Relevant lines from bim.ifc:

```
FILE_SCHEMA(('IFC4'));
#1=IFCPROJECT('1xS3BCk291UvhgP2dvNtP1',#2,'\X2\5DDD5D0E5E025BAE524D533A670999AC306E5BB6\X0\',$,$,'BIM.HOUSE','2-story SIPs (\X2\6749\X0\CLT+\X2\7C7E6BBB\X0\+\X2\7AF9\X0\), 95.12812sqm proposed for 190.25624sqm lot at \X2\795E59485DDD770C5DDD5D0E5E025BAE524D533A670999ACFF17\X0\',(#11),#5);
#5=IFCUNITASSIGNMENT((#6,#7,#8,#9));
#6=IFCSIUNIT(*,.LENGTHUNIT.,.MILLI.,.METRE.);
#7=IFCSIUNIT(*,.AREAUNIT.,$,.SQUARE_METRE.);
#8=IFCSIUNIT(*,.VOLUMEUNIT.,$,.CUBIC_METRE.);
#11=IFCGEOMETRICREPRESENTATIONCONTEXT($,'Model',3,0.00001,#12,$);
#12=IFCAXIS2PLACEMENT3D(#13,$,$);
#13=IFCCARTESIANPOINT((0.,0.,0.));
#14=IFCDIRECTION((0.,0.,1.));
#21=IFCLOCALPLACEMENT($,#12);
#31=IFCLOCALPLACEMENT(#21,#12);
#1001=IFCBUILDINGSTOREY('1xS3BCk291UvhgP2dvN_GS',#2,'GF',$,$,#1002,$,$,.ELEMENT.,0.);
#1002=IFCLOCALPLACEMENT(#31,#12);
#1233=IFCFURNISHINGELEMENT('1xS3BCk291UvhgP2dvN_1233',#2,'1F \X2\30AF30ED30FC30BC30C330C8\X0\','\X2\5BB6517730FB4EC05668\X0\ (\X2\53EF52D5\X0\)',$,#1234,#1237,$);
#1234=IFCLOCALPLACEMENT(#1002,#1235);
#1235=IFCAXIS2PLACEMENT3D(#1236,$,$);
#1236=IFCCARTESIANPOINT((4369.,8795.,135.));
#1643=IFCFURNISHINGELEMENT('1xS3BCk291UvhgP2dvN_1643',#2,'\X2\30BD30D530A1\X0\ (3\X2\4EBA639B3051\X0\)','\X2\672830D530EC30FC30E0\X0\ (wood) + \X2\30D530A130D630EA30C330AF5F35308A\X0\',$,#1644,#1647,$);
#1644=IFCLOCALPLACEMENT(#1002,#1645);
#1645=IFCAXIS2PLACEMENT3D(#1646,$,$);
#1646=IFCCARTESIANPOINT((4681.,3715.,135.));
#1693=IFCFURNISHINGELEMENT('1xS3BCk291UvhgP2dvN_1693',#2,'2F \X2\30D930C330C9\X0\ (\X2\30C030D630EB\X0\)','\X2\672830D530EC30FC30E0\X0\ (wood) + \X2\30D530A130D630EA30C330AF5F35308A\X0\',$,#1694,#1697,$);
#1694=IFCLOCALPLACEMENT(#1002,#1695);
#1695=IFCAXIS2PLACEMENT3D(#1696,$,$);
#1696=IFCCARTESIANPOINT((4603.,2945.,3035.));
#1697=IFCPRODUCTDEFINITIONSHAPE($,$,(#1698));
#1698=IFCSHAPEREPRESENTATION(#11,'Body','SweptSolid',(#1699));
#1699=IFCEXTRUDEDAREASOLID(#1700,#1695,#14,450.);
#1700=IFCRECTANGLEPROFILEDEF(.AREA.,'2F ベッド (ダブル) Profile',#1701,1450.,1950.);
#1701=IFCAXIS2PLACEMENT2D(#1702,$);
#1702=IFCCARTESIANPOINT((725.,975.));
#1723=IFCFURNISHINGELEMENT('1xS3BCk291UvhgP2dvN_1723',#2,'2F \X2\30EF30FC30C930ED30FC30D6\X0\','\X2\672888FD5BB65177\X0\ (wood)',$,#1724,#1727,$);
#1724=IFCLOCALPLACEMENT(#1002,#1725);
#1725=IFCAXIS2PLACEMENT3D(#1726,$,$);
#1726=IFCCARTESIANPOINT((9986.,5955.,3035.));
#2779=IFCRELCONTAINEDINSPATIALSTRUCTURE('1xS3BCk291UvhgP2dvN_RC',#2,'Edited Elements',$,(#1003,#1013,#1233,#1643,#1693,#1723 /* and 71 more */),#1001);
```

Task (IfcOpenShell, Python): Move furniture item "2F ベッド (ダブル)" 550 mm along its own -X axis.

```python
import ifcopenshell
import ifcopenshell.api.geometry
import ifcopenshell.util.placement
import ifcopenshell.util.unit

model = ifcopenshell.open("bim.ifc")
unit_scale = ifcopenshell.util.unit.calculate_unit_scale(model)

item = model.by_guid("1xS3BCk291UvhgP2dvN_1693")
matrix = ifcopenshell.util.placement.get_local_placement(item.ObjectPlacement)
matrix[:3, 3] -= matrix[:3, 0] * 0.55 / unit_scale
ifcopenshell.api.geometry.edit_object_placement(model, product=item, matrix=matrix, is_si=False)

print(ifcopenshell.util.placement.get_local_placement(item.ObjectPlacement).round(3) + 0.0)

model.write("bim_rev.ifc")
```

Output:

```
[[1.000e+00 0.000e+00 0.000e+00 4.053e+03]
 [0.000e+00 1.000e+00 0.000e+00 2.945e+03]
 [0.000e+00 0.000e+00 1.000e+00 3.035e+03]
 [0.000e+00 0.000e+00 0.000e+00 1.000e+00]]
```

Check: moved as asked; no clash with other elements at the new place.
